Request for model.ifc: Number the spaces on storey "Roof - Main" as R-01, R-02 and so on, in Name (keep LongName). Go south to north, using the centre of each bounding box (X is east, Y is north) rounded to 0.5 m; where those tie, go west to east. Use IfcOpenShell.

First a look at what the model holds.

```python
import ifcopenshell
import ifcopenshell.util.element
import ifcopenshell.util.placement

model = ifcopenshell.open("model.ifc")
print(model.schema)
storey = next(s for s in model.by_type("IfcBuildingStorey") if s.Name == "Roof - Main")
spaces = [e for e in ifcopenshell.util.element.get_decomposition(storey) if e.is_a("IfcSpace")]
for e in sorted(spaces, key=lambda e: e.id()):
    origin = ifcopenshell.util.placement.get_local_placement(e.ObjectPlacement)[:3, 3]
    print(e.id(), e.Name, e.LongName, origin.round(2) + 0.0, sep=" | ")
```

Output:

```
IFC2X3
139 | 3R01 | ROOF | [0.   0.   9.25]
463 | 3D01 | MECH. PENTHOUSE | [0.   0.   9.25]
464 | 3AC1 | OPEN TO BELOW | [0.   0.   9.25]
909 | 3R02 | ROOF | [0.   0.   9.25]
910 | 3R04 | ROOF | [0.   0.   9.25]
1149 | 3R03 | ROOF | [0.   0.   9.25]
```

```python
import ifcopenshell
import ifcopenshell.geom
import ifcopenshell.util.element
import ifcopenshell.util.shape

model = ifcopenshell.open("model.ifc")
settings = ifcopenshell.geom.settings()
settings.set("use-world-coords", True)


def centre(element):
    shape = ifcopenshell.geom.create_shape(settings, element)
    return ifcopenshell.util.shape.get_bbox_centroid(shape.geometry)


storey = next(s for s in model.by_type("IfcBuildingStorey") if s.Name == "Roof - Main")
spaces = [e for e in ifcopenshell.util.element.get_decomposition(storey) if e.is_a("IfcSpace")]

# Insertion points can sit at a corner or the storey origin, so sort by the geometry (in metres).
centres = {e: centre(e) for e in spaces}
spaces.sort(key=lambda e: (round(centres[e][1] / 0.5), centres[e][0]))

for i, e in enumerate(spaces, start=1):
    number = f"R-{i:02d}"
    e.Name = number
    print(e.id(), number)

model.write("model_v2.ifc")
```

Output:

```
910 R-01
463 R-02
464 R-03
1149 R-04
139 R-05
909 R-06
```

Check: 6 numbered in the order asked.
